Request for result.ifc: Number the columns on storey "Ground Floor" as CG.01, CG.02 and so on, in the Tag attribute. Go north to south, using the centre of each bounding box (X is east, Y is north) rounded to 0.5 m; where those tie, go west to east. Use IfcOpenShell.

First a look at what the model holds.

```python
import ifcopenshell
import ifcopenshell.util.element
import ifcopenshell.util.placement

model = ifcopenshell.open("result.ifc")
print(model.schema)
storey = next(s for s in model.by_type("IfcBuildingStorey") if s.Name == "Ground Floor")
columns = [e for e in ifcopenshell.util.element.get_decomposition(storey) if e.is_a("IfcColumn")]
for e in sorted(columns, key=lambda e: e.id()):
    origin = ifcopenshell.util.placement.get_local_placement(e.ObjectPlacement)[:3, 3]
    print(e.id(), e.Tag, e.Name, origin.round(2) + 0.0, sep=" | ")
```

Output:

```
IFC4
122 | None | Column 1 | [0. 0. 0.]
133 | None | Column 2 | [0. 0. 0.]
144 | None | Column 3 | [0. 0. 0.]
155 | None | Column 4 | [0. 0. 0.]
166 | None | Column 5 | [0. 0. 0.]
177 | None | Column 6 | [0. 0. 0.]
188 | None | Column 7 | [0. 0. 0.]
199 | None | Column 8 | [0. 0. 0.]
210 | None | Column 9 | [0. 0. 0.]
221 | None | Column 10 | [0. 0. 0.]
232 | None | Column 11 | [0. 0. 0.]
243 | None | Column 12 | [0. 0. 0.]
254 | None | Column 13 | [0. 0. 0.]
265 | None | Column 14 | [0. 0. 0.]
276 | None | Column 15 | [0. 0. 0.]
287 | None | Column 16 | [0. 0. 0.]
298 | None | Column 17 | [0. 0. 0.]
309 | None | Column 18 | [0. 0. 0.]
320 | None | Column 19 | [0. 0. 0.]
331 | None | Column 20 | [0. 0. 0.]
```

```python
import ifcopenshell
import ifcopenshell.geom
import ifcopenshell.util.element
import ifcopenshell.util.shape

model = ifcopenshell.open("result.ifc")
settings = ifcopenshell.geom.settings()
settings.set("use-world-coords", True)


def centre(element):
    shape = ifcopenshell.geom.create_shape(settings, element)
    return ifcopenshell.util.shape.get_bbox_centroid(shape.geometry)


storey = next(s for s in model.by_type("IfcBuildingStorey") if s.Name == "Ground Floor")
columns = [e for e in ifcopenshell.util.element.get_decomposition(storey) if e.is_a("IfcColumn")]

# Insertion points can sit at a corner or the storey origin, so sort by the geometry (in metres).
centres = {e: centre(e) for e in columns}
columns.sort(key=lambda e: (-round(centres[e][1] / 0.5), centres[e][0]))

for i, e in enumerate(columns, start=1):
    number = f"CG.{i:02d}"
    e.Tag = number
    print(e.id(), number)

model.write("result_v2.ifc")
```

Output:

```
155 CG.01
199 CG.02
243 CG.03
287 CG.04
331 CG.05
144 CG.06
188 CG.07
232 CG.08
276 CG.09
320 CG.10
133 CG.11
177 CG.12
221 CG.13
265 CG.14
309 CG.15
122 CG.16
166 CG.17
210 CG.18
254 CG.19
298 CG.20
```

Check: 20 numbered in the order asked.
